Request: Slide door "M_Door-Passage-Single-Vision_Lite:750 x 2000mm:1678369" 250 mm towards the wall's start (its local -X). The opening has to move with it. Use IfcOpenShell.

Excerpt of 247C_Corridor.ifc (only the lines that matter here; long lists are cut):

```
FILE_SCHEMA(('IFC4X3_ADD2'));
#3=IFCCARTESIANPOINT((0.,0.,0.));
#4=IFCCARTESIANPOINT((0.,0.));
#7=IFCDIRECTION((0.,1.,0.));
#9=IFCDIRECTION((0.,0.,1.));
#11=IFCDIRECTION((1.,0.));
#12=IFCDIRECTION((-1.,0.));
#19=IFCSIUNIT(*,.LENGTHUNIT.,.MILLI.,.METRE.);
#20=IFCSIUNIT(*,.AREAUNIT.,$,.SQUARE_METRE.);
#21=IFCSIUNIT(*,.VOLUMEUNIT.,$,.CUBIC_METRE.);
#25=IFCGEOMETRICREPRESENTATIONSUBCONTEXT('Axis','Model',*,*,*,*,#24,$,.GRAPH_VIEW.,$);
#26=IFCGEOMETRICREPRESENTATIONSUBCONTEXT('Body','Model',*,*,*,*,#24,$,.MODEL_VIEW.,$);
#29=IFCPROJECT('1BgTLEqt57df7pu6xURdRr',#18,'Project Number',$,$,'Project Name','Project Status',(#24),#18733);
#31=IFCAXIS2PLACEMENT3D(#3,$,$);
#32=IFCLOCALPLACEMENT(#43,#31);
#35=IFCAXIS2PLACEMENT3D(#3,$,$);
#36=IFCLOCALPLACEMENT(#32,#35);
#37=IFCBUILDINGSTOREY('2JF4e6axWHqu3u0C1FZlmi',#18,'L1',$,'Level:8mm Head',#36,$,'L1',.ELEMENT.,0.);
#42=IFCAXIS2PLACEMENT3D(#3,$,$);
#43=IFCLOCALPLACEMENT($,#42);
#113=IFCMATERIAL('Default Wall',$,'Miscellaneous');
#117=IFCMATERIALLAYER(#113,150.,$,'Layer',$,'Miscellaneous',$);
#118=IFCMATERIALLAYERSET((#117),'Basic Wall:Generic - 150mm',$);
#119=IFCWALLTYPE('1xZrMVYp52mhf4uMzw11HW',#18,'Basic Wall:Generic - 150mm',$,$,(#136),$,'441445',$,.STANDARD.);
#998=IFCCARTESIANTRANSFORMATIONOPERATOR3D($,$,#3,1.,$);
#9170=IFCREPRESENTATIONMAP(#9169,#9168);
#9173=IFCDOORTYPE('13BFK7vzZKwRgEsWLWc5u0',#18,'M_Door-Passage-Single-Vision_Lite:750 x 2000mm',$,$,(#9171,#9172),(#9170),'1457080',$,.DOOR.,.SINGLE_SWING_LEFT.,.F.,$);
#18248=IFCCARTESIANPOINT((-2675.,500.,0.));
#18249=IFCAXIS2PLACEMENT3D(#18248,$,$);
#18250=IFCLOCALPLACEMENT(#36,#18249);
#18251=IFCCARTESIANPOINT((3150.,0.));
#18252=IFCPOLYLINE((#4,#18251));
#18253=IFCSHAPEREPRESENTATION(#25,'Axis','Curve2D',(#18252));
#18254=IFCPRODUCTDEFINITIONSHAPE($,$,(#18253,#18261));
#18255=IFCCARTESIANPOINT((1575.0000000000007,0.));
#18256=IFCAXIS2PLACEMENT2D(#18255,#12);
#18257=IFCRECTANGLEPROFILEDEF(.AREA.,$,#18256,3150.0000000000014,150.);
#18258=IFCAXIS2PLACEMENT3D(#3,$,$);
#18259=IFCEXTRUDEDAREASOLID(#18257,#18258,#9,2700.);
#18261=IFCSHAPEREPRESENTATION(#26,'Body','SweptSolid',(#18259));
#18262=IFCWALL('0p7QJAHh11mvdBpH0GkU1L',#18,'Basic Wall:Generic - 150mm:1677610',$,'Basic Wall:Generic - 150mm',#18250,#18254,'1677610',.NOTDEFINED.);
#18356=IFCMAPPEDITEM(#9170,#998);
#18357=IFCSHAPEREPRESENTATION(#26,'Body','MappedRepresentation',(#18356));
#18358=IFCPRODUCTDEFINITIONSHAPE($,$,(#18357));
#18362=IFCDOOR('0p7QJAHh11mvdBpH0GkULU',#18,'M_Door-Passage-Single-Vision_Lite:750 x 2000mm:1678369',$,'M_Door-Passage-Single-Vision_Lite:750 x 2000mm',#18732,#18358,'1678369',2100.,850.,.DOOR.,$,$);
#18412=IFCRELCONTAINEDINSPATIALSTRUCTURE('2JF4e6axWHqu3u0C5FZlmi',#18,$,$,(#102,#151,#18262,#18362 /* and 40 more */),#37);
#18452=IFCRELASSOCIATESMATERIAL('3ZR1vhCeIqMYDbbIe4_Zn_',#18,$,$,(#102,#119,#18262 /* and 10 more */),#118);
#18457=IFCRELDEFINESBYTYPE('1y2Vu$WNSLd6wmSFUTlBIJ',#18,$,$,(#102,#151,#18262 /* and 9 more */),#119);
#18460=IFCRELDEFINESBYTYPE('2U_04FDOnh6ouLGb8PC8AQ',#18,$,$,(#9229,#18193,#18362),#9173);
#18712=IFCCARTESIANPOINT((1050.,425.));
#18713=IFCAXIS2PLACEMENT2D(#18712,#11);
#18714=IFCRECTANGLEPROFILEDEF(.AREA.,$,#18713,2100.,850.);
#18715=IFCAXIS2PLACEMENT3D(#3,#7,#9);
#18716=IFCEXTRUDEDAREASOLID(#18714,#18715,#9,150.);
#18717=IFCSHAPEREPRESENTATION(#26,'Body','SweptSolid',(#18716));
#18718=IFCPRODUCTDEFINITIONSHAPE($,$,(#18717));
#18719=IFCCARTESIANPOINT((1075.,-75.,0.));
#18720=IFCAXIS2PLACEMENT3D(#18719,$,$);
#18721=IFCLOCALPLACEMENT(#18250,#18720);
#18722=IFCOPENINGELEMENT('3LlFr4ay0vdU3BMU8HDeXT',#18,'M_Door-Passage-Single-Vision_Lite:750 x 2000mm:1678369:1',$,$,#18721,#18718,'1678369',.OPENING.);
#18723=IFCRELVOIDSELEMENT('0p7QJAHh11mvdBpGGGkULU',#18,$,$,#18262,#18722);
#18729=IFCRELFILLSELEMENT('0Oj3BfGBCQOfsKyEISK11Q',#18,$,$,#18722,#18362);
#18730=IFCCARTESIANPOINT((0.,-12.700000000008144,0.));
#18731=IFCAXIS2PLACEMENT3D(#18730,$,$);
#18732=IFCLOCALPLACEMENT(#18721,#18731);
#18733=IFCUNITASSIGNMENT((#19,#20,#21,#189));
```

```python
import ifcopenshell
import ifcopenshell.api.geometry
import ifcopenshell.util.placement

model = ifcopenshell.open("247C_Corridor.ifc")

door = model.by_guid("0p7QJAHh11mvdBpH0GkULU")
opening = door.FillsVoids[0].RelatingOpeningElement
wall = opening.VoidsElements[0].RelatingBuildingElement

wall_matrix = ifcopenshell.util.placement.get_local_placement(wall.ObjectPlacement)
shift = wall_matrix[:3, 0] * -250.0
before = ifcopenshell.util.placement.get_local_placement(door.ObjectPlacement)[:3, 3].copy()

# The door is placed relative to its opening, so it follows when the opening moves.
matrix = ifcopenshell.util.placement.get_local_placement(opening.ObjectPlacement)
matrix[:3, 3] += shift
ifcopenshell.api.geometry.edit_object_placement(
    model, product=opening, matrix=matrix, is_si=False, should_transform_children=True
)

after = ifcopenshell.util.placement.get_local_placement(door.ObjectPlacement)[:3, 3]
print("door moved by", (after - before).round(3) + 0.0)

model.write("247C_Corridor_rev.ifc")
```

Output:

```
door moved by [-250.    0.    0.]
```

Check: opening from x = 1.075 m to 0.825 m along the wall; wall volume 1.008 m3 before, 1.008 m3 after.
